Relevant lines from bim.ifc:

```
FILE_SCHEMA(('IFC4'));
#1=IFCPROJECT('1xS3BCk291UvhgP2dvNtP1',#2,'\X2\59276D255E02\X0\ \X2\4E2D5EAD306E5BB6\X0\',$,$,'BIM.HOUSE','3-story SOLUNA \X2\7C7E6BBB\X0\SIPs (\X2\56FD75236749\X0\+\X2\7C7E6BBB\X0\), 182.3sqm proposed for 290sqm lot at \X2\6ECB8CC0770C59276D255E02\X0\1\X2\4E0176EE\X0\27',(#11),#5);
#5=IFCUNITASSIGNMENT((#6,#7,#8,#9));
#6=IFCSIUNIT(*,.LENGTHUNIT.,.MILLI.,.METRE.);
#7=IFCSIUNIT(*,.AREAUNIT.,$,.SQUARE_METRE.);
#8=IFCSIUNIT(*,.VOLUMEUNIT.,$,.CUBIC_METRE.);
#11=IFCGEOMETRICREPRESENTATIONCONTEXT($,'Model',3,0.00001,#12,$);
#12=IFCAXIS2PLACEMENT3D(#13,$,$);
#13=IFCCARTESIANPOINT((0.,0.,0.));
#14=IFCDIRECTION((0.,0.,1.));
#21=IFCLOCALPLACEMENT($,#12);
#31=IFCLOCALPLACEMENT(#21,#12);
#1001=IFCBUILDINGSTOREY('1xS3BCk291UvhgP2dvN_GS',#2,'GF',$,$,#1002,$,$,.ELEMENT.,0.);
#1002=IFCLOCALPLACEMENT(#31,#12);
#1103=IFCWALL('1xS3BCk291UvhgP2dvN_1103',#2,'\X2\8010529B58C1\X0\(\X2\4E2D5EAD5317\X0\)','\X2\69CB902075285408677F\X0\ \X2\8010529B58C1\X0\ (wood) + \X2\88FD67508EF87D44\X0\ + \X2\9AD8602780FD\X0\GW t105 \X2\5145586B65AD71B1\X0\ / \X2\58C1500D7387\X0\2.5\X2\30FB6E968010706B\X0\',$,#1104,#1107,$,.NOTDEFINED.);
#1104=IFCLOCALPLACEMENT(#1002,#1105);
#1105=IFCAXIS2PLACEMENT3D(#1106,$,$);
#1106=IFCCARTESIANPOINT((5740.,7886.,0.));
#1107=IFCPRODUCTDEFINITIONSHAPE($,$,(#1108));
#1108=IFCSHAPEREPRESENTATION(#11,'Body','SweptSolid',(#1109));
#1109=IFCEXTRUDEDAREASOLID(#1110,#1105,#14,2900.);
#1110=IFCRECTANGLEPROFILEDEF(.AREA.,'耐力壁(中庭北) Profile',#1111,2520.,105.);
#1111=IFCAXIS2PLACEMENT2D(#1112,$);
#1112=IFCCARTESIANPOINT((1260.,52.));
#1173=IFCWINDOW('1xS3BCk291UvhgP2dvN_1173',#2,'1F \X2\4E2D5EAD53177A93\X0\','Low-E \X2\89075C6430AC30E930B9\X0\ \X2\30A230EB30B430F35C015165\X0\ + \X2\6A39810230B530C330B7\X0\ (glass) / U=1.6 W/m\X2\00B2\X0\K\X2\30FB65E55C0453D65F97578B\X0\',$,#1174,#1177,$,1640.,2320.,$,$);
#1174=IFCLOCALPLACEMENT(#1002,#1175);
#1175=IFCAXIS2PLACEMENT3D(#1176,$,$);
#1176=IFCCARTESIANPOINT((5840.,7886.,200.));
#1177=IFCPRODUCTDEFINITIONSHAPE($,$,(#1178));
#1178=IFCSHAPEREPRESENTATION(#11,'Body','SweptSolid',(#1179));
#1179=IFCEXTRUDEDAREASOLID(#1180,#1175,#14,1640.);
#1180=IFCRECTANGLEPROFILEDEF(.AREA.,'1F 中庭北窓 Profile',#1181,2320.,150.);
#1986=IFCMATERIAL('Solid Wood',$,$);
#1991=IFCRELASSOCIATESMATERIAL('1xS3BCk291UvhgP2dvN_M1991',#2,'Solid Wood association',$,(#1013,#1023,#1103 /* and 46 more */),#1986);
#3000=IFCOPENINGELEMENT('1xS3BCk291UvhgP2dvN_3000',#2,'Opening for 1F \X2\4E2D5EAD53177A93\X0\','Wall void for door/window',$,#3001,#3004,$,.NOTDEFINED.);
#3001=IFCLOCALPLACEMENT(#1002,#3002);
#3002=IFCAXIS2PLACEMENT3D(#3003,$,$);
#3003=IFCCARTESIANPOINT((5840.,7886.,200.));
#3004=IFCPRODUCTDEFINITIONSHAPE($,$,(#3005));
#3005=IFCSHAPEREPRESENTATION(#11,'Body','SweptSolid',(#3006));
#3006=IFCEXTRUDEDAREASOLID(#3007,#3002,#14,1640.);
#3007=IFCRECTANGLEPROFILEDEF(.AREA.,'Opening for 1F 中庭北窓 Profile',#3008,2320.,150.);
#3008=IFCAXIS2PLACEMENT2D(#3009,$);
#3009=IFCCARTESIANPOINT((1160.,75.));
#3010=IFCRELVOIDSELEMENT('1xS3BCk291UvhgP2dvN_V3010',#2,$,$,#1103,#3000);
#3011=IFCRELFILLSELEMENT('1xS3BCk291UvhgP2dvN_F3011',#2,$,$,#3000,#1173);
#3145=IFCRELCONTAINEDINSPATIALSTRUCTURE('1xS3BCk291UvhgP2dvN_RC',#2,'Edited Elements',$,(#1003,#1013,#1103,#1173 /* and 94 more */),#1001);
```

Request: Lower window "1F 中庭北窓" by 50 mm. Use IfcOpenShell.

```python
import numpy as np
import ifcopenshell
import ifcopenshell.api.geometry
import ifcopenshell.util.placement
import ifcopenshell.util.unit

model = ifcopenshell.open("bim.ifc")
unit_scale = ifcopenshell.util.unit.calculate_unit_scale(model)

window = model.by_guid("1xS3BCk291UvhgP2dvN_1173")
opening = window.FillsVoids[0].RelatingOpeningElement
dz = -0.05 / unit_scale

shift = np.array([0.0, 0.0, dz])
# The window is not placed relative to its opening, so move both.
for product in (opening, window):
    matrix = ifcopenshell.util.placement.get_local_placement(product.ObjectPlacement)
    matrix[:3, 3] += shift
    ifcopenshell.api.geometry.edit_object_placement(model, product=product, matrix=matrix, is_si=False)

print(f"moved by {dz * unit_scale:+.3f} m")

model.write("bim_v2.ifc")
```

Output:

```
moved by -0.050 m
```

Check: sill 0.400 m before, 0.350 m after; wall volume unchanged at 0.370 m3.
